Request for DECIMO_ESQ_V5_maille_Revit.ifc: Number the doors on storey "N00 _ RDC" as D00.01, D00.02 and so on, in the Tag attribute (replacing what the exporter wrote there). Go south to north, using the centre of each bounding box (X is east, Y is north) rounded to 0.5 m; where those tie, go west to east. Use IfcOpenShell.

First a look at what the model holds.

```python
import ifcopenshell
import ifcopenshell.util.element
import ifcopenshell.util.placement

model = ifcopenshell.open("DECIMO_ESQ_V5_maille_Revit.ifc")
print(model.schema)
storey = next(s for s in model.by_type("IfcBuildingStorey") if s.Name == "N00 _ RDC")
doors = [e for e in ifcopenshell.util.element.get_decomposition(storey) if e.is_a("IfcDoor")]
for e in sorted(doors, key=lambda e: e.id()):
    origin = ifcopenshell.util.placement.get_local_placement(e.ObjectPlacement)[:3, 3]
    print(e.id(), e.Tag, e.Name, origin.round(2) + 0.0, sep=" | ")
```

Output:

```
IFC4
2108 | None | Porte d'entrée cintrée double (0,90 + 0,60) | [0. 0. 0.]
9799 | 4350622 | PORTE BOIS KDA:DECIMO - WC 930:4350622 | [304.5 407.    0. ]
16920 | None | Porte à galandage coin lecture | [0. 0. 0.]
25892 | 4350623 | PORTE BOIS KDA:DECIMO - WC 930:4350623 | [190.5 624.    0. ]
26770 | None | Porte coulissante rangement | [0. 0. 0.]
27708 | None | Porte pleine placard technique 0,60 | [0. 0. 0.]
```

```python
import ifcopenshell
import ifcopenshell.geom
import ifcopenshell.util.element
import ifcopenshell.util.shape

model = ifcopenshell.open("DECIMO_ESQ_V5_maille_Revit.ifc")
settings = ifcopenshell.geom.settings()
settings.set("use-world-coords", True)


def centre(element):
    shape = ifcopenshell.geom.create_shape(settings, element)
    return ifcopenshell.util.shape.get_bbox_centroid(shape.geometry)


storey = next(s for s in model.by_type("IfcBuildingStorey") if s.Name == "N00 _ RDC")
doors = [e for e in ifcopenshell.util.element.get_decomposition(storey) if e.is_a("IfcDoor")]

# Insertion points can sit at a corner or the storey origin, so sort by the geometry (in metres).
centres = {e: centre(e) for e in doors}
doors.sort(key=lambda e: (round(centres[e][1] / 0.5), centres[e][0]))

for i, e in enumerate(doors, start=1):
    number = f"D00.{i:02d}"
    e.Tag = number
    print(e.id(), number)

model.write("DECIMO_ESQ_V5_maille_Revit_edited.ifc")
```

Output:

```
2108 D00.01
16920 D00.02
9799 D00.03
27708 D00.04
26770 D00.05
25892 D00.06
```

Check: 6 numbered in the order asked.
